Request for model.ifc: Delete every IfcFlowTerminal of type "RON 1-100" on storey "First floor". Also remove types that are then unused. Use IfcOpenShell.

First a look at what the model holds.

```python
import ifcopenshell
import ifcopenshell.util.element

model = ifcopenshell.open("model.ifc")
print(model.schema)
storey = next(s for s in model.by_type("IfcBuildingStorey") if s.Name == "First floor")
terminals = [e for e in ifcopenshell.util.element.get_decomposition(storey) if e.is_a("IfcFlowTerminal")]
seen = {}
for e in terminals:
    element_type = ifcopenshell.util.element.get_type(e)
    name = element_type.Name if element_type not in (None, e) else None
    seen[name] = seen.get(name, 0) + 1
for name, count in sorted(seen.items(), key=str):
    print(count, "x", name)
```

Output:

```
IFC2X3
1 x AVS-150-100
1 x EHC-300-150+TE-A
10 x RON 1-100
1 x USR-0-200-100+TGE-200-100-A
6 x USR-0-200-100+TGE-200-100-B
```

```python
import ifcopenshell
import ifcopenshell.api.root
import ifcopenshell.util.element

model = ifcopenshell.open("model.ifc")

storey = next(s for s in model.by_type("IfcBuildingStorey") if s.Name == "First floor")
terminals = [e for e in ifcopenshell.util.element.get_decomposition(storey) if e.is_a("IfcFlowTerminal")]
targets = [e for e in terminals if (t := ifcopenshell.util.element.get_type(e)) not in (None, e) and t.Name == "RON 1-100"]
types = {ifcopenshell.util.element.get_type(e) for e in targets} - {None, *targets}

for e in targets:
    ifcopenshell.api.root.remove_product(model, product=e)
print(len(targets), "removed")

unused = [t for t in types if not ifcopenshell.util.element.get_types(t)]
for t in unused:
    ifcopenshell.api.root.remove_product(model, product=t)
print(len(unused), "unused types removed")

model.write("model-out.ifc")
```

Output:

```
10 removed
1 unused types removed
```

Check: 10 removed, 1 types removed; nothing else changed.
